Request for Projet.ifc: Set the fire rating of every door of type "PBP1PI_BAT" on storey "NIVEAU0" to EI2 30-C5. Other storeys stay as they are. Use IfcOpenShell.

First a look at what the model holds.

```python
import ifcopenshell
import ifcopenshell.util.element

model = ifcopenshell.open("Projet.ifc")
print(model.schema)
storey = next(s for s in model.by_type("IfcBuildingStorey") if s.Name == "NIVEAU0")
doors = [e for e in ifcopenshell.util.element.get_decomposition(storey) if e.is_a("IfcDoor")]
seen = {}
for e in doors:
    element_type = ifcopenshell.util.element.get_type(e)
    key = (element_type.Name if element_type != e and element_type else None, ifcopenshell.util.element.get_pset(e, "Pset_DoorCommon", "FireRating"))
    seen[key] = seen.get(key, 0) + 1
for (name, value), count in sorted(seen.items(), key=str):
    print(count, "x", name, "|", value)
```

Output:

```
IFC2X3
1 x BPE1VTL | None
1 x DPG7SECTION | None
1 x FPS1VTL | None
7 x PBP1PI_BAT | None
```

```python
import ifcopenshell
import ifcopenshell.api.pset
import ifcopenshell.util.element

model = ifcopenshell.open("Projet.ifc")

storey = next(s for s in model.by_type("IfcBuildingStorey") if s.Name == "NIVEAU0")
doors = [e for e in ifcopenshell.util.element.get_decomposition(storey) if e.is_a("IfcDoor")]

count = 0
for e in doors:
    element_type = ifcopenshell.util.element.get_type(e)
    if element_type in (None, e) or element_type.Name != "PBP1PI_BAT":
        continue
    # add_pset returns the element's existing set when there is one.
    pset = ifcopenshell.api.pset.add_pset(model, product=e, name="Pset_DoorCommon")
    ifcopenshell.api.pset.edit_pset(model, pset=pset, properties={"FireRating": "EI2 30-C5"})
    count += 1

print(count, "doors updated")

model.write("Projet_updated.ifc")
```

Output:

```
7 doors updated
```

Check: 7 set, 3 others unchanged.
